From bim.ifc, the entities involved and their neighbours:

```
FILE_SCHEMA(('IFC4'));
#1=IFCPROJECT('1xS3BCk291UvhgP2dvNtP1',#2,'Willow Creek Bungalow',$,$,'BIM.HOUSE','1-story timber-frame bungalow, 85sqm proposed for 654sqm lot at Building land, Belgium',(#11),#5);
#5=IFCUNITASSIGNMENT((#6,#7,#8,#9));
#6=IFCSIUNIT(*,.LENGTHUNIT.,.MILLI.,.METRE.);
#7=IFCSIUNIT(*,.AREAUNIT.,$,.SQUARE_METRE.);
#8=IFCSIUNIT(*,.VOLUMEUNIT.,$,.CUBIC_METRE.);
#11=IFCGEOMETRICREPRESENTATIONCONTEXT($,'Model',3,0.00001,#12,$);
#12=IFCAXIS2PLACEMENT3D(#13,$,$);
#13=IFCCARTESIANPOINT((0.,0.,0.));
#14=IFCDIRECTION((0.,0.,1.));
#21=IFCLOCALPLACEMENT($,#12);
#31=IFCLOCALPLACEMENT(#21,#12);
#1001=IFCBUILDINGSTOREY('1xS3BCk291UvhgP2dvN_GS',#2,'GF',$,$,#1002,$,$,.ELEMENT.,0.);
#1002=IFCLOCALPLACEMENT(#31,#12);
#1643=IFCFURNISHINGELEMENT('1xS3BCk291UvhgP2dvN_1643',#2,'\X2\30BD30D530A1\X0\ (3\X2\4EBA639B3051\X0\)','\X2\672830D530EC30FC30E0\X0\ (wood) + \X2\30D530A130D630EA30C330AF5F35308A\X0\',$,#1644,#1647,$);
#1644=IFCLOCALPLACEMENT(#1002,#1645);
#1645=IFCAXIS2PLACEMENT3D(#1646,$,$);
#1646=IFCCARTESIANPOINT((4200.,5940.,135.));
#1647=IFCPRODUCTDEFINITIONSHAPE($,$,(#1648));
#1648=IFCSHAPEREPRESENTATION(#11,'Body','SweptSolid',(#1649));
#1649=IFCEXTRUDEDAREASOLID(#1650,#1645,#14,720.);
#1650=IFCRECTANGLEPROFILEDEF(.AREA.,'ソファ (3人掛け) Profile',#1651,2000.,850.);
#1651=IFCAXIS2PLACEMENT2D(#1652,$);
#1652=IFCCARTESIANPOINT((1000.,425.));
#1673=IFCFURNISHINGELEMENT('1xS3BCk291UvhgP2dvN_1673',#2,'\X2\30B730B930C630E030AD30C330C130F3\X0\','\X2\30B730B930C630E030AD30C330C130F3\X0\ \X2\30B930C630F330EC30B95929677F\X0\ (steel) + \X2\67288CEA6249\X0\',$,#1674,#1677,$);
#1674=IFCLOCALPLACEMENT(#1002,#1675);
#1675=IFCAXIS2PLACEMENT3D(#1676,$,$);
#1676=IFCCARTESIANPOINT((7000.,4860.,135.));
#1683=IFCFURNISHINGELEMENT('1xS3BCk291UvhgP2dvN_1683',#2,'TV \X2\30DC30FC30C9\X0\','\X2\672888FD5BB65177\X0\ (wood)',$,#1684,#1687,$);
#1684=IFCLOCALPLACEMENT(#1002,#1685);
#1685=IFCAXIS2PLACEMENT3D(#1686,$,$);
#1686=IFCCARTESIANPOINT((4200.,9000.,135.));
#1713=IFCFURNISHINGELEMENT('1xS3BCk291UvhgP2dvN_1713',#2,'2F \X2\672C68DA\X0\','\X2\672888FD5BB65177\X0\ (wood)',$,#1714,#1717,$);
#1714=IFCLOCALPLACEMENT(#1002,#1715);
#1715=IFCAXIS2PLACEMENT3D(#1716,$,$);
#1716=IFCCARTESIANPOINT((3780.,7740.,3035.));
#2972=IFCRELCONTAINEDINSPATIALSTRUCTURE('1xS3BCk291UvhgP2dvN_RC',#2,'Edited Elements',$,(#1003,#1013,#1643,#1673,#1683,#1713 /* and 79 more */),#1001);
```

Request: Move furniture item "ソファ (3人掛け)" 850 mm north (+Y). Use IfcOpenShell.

```python
import ifcopenshell
import ifcopenshell.api.geometry
import ifcopenshell.util.placement
import ifcopenshell.util.unit

model = ifcopenshell.open("bim.ifc")
unit_scale = ifcopenshell.util.unit.calculate_unit_scale(model)

item = model.by_id(1643)
matrix = ifcopenshell.util.placement.get_local_placement(item.ObjectPlacement)
matrix[1, 3] += 0.85 / unit_scale
ifcopenshell.api.geometry.edit_object_placement(model, product=item, matrix=matrix, is_si=False)

print(ifcopenshell.util.placement.get_local_placement(item.ObjectPlacement).round(3) + 0.0)

model.write("bim-out.ifc")
```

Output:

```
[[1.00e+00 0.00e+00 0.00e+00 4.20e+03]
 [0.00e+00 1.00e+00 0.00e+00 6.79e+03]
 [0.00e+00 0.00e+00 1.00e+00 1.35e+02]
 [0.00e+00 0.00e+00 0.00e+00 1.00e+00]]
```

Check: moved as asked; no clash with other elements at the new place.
